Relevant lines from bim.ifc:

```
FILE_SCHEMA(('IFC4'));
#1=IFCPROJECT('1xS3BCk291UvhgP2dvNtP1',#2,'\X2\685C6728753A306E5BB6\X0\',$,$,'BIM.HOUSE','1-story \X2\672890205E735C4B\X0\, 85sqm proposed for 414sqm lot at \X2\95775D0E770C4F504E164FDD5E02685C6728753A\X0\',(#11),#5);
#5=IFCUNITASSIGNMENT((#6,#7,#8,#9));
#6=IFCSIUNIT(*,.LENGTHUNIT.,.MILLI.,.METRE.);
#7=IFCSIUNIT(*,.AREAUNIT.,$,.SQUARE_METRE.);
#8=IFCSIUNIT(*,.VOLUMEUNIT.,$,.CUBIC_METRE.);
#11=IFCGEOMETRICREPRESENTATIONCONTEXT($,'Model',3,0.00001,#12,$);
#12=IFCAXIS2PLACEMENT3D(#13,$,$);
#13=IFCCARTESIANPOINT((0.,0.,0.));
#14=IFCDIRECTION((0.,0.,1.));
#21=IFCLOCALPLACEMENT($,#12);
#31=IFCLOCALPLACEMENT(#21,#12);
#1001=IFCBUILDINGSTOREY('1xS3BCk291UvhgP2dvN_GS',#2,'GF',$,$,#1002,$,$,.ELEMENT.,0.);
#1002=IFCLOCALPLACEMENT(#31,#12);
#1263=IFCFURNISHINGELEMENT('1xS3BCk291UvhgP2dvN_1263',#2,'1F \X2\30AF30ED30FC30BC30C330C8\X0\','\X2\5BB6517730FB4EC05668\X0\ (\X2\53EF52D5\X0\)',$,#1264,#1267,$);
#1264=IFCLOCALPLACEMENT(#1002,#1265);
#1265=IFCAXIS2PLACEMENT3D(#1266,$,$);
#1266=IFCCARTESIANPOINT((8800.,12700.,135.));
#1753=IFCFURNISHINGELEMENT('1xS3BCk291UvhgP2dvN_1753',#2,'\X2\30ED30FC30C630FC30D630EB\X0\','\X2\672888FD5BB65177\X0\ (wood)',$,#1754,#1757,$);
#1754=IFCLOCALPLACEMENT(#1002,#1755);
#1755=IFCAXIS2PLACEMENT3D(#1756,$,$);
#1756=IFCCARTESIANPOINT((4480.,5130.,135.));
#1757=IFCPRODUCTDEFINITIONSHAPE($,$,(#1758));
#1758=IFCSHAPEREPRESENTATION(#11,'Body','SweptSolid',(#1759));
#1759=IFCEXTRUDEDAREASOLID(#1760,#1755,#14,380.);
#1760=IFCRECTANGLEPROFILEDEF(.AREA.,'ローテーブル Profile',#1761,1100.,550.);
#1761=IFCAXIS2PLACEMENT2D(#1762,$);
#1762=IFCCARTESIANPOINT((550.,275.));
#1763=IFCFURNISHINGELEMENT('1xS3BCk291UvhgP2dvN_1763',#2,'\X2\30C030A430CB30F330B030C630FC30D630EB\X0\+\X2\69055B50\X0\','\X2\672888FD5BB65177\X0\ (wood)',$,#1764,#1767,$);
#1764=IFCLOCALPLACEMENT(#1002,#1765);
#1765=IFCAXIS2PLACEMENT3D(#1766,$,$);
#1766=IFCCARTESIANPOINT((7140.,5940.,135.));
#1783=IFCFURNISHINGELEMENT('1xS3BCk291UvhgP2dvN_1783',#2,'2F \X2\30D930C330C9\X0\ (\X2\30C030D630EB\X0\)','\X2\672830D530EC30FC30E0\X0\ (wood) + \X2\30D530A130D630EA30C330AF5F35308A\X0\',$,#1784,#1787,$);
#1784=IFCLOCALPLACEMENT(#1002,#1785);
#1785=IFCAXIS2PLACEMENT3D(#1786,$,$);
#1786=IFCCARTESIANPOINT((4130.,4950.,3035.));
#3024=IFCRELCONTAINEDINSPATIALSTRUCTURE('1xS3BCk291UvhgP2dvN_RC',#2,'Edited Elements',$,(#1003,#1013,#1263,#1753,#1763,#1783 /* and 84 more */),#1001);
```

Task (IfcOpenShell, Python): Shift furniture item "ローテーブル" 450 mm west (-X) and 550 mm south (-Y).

```python
import ifcopenshell
import ifcopenshell.api.geometry
import ifcopenshell.util.placement
import ifcopenshell.util.unit

model = ifcopenshell.open("bim.ifc")
unit_scale = ifcopenshell.util.unit.calculate_unit_scale(model)

item = model.by_guid("1xS3BCk291UvhgP2dvN_1753")
matrix = ifcopenshell.util.placement.get_local_placement(item.ObjectPlacement)
matrix[0, 3] -= 0.45 / unit_scale
matrix[1, 3] -= 0.55 / unit_scale
ifcopenshell.api.geometry.edit_object_placement(model, product=item, matrix=matrix, is_si=False)

print(ifcopenshell.util.placement.get_local_placement(item.ObjectPlacement).round(3) + 0.0)

model.write("bim_edited.ifc")
```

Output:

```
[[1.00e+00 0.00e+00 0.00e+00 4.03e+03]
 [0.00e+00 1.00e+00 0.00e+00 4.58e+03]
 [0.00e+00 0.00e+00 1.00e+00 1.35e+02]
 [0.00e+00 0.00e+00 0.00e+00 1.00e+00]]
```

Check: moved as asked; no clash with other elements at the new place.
